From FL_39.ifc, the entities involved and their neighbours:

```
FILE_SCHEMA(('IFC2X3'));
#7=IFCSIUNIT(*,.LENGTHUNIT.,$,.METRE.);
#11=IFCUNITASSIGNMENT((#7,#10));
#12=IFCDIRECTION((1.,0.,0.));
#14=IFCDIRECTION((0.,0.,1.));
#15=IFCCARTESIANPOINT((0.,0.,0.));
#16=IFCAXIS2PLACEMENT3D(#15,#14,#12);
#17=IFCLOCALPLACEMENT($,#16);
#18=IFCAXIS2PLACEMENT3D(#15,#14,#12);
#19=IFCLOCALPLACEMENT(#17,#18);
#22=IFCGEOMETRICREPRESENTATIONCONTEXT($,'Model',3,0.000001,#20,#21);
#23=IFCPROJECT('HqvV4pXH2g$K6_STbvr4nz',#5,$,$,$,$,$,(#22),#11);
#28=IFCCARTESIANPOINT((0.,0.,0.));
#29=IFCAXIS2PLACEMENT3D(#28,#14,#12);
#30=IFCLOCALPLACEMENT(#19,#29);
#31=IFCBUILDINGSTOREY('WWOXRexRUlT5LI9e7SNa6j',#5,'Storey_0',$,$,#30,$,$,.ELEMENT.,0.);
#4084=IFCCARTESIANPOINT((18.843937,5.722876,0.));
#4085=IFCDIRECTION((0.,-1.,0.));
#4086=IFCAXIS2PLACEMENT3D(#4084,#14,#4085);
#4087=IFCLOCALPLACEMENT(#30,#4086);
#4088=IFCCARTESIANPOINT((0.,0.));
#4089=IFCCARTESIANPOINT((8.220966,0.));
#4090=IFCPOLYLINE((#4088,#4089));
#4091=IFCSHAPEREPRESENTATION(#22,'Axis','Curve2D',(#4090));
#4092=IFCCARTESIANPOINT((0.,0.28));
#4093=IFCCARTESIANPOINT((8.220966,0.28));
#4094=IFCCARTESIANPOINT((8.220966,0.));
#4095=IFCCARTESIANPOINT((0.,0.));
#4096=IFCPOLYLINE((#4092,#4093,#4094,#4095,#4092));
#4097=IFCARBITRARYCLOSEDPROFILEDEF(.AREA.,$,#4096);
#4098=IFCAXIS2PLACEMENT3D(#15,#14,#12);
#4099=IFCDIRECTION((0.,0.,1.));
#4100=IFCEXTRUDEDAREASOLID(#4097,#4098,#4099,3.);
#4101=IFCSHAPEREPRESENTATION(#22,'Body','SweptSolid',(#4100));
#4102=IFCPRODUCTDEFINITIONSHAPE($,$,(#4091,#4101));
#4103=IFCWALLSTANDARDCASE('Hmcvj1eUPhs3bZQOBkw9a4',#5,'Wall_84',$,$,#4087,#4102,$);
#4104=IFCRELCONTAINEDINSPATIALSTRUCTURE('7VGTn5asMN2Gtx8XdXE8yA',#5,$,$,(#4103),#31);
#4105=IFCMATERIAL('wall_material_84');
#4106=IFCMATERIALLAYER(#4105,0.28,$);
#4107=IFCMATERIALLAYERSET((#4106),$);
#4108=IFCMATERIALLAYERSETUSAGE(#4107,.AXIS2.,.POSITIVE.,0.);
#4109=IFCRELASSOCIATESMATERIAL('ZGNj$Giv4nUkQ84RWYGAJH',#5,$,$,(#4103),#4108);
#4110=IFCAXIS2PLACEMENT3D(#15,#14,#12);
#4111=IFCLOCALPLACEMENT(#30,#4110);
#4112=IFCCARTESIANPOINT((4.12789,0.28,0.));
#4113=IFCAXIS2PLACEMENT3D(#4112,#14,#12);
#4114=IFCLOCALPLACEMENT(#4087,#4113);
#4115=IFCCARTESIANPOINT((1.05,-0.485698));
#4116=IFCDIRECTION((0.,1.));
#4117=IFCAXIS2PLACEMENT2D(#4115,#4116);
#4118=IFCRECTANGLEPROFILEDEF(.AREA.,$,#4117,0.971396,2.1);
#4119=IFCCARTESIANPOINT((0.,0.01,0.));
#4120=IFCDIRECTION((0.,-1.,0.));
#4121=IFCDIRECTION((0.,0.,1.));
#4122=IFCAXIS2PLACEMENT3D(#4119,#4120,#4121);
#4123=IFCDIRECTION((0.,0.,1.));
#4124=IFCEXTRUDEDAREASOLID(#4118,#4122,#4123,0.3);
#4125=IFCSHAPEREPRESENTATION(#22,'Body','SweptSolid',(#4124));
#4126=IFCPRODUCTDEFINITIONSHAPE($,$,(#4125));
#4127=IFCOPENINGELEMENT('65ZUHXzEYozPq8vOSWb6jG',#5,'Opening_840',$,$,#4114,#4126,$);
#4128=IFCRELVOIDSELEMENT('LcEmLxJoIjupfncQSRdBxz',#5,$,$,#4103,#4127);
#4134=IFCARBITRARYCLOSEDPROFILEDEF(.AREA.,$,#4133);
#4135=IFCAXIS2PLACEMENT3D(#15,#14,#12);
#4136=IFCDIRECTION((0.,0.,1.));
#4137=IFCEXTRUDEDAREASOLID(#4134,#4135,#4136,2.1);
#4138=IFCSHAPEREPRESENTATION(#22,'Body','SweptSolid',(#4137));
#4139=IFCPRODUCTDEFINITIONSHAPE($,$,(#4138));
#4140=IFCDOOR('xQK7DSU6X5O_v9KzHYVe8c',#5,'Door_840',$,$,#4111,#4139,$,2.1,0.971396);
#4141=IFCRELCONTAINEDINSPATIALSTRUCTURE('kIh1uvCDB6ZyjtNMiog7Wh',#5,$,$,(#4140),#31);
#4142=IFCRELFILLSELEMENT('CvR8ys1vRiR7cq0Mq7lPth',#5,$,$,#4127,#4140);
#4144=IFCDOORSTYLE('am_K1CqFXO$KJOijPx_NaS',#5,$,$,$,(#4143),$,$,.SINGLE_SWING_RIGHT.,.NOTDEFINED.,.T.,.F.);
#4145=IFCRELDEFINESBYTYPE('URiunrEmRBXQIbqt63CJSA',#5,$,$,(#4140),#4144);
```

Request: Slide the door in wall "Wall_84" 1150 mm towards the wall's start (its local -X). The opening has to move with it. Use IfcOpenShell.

```python
import ifcopenshell
import ifcopenshell.api.geometry
import ifcopenshell.util.placement
import ifcopenshell.util.unit

model = ifcopenshell.open("FL_39.ifc")
unit_scale = ifcopenshell.util.unit.calculate_unit_scale(model)

door = model.by_guid("xQK7DSU6X5O_v9KzHYVe8c")
opening = door.FillsVoids[0].RelatingOpeningElement
wall = opening.VoidsElements[0].RelatingBuildingElement

wall_matrix = ifcopenshell.util.placement.get_local_placement(wall.ObjectPlacement)
shift = wall_matrix[:3, 0] * -1.15 / unit_scale
before = ifcopenshell.util.placement.get_local_placement(door.ObjectPlacement)[:3, 3].copy()

# The door is not placed relative to its opening, so move both.
for product in (opening, door):
    matrix = ifcopenshell.util.placement.get_local_placement(product.ObjectPlacement)
    matrix[:3, 3] += shift
    ifcopenshell.api.geometry.edit_object_placement(model, product=product, matrix=matrix, is_si=False)

after = ifcopenshell.util.placement.get_local_placement(door.ObjectPlacement)[:3, 3]
print("door moved by", (after - before).round(3) + 0.0)

model.write("FL_39-out.ifc")
```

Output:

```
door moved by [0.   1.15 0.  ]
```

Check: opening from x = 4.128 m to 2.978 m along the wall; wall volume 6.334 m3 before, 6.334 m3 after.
